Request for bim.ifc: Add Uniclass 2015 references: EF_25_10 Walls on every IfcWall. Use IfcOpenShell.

First a look at what the model holds.

```python
import ifcopenshell

model = ifcopenshell.open("bim.ifc")
print(model.schema)
print("classifications:", [c.Name for c in model.by_type("IfcClassification")])
for ifc_class in ("IfcDoor", "IfcRoof", "IfcStair", "IfcWall", "IfcWindow"):
    print(ifc_class, len(model.by_type(ifc_class)))
```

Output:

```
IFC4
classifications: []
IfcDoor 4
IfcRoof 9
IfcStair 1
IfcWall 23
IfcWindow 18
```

```python
import ifcopenshell
import ifcopenshell.api.classification

model = ifcopenshell.open("bim.ifc")

system = ifcopenshell.api.classification.add_classification(model, classification="Uniclass 2015")

codes = {
    "IfcWall": ("EF_25_10", "Walls"),
}
for ifc_class, (code, name) in codes.items():
    products = model.by_type(ifc_class)
    ifcopenshell.api.classification.add_reference(
        model, products=products, classification=system, identification=code, name=name
    )
    print(code, len(products))

model.write("bim_rev.ifc")
```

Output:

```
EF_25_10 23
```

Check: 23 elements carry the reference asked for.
